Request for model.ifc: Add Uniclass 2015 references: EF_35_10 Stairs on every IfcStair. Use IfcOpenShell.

First a look at what the model holds.

```python
import ifcopenshell

model = ifcopenshell.open("model.ifc")
print(model.schema)
print("classifications:", [c.Name for c in model.by_type("IfcClassification")])
for ifc_class in ("IfcDoor", "IfcRoof", "IfcStair", "IfcWall", "IfcWindow"):
    print(ifc_class, len(model.by_type(ifc_class)))
```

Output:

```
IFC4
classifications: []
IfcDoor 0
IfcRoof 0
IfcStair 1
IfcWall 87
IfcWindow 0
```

```python
import ifcopenshell
import ifcopenshell.api.classification

model = ifcopenshell.open("model.ifc")

system = ifcopenshell.api.classification.add_classification(model, classification="Uniclass 2015")

codes = {
    "IfcStair": ("EF_35_10", "Stairs"),
}
for ifc_class, (code, name) in codes.items():
    products = model.by_type(ifc_class)
    ifcopenshell.api.classification.add_reference(
        model, products=products, classification=system, identification=code, name=name
    )
    print(code, len(products))

model.write("model_edited.ifc")
```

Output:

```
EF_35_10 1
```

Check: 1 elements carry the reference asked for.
